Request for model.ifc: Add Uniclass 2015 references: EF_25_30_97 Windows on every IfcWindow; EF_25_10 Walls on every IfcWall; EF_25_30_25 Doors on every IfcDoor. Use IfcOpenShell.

First a look at what the model holds.

```python
import ifcopenshell

model = ifcopenshell.open("model.ifc")
print(model.schema)
print("classifications:", [c.Name for c in model.by_type("IfcClassification")])
for ifc_class in ("IfcDoor", "IfcRoof", "IfcStair", "IfcWall", "IfcWindow"):
    print(ifc_class, len(model.by_type(ifc_class)))
```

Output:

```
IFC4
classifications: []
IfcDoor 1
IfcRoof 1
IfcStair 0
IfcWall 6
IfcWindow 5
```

```python
import ifcopenshell
import ifcopenshell.api.classification

model = ifcopenshell.open("model.ifc")

system = ifcopenshell.api.classification.add_classification(model, classification="Uniclass 2015")

codes = {
    "IfcWindow": ("EF_25_30_97", "Windows"),
    "IfcWall": ("EF_25_10", "Walls"),
    "IfcDoor": ("EF_25_30_25", "Doors"),
}
for ifc_class, (code, name) in codes.items():
    products = model.by_type(ifc_class)
    ifcopenshell.api.classification.add_reference(
        model, products=products, classification=system, identification=code, name=name
    )
    print(code, len(products))

model.write("model_rev.ifc")
```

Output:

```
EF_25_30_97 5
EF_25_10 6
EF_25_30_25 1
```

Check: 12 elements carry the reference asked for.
